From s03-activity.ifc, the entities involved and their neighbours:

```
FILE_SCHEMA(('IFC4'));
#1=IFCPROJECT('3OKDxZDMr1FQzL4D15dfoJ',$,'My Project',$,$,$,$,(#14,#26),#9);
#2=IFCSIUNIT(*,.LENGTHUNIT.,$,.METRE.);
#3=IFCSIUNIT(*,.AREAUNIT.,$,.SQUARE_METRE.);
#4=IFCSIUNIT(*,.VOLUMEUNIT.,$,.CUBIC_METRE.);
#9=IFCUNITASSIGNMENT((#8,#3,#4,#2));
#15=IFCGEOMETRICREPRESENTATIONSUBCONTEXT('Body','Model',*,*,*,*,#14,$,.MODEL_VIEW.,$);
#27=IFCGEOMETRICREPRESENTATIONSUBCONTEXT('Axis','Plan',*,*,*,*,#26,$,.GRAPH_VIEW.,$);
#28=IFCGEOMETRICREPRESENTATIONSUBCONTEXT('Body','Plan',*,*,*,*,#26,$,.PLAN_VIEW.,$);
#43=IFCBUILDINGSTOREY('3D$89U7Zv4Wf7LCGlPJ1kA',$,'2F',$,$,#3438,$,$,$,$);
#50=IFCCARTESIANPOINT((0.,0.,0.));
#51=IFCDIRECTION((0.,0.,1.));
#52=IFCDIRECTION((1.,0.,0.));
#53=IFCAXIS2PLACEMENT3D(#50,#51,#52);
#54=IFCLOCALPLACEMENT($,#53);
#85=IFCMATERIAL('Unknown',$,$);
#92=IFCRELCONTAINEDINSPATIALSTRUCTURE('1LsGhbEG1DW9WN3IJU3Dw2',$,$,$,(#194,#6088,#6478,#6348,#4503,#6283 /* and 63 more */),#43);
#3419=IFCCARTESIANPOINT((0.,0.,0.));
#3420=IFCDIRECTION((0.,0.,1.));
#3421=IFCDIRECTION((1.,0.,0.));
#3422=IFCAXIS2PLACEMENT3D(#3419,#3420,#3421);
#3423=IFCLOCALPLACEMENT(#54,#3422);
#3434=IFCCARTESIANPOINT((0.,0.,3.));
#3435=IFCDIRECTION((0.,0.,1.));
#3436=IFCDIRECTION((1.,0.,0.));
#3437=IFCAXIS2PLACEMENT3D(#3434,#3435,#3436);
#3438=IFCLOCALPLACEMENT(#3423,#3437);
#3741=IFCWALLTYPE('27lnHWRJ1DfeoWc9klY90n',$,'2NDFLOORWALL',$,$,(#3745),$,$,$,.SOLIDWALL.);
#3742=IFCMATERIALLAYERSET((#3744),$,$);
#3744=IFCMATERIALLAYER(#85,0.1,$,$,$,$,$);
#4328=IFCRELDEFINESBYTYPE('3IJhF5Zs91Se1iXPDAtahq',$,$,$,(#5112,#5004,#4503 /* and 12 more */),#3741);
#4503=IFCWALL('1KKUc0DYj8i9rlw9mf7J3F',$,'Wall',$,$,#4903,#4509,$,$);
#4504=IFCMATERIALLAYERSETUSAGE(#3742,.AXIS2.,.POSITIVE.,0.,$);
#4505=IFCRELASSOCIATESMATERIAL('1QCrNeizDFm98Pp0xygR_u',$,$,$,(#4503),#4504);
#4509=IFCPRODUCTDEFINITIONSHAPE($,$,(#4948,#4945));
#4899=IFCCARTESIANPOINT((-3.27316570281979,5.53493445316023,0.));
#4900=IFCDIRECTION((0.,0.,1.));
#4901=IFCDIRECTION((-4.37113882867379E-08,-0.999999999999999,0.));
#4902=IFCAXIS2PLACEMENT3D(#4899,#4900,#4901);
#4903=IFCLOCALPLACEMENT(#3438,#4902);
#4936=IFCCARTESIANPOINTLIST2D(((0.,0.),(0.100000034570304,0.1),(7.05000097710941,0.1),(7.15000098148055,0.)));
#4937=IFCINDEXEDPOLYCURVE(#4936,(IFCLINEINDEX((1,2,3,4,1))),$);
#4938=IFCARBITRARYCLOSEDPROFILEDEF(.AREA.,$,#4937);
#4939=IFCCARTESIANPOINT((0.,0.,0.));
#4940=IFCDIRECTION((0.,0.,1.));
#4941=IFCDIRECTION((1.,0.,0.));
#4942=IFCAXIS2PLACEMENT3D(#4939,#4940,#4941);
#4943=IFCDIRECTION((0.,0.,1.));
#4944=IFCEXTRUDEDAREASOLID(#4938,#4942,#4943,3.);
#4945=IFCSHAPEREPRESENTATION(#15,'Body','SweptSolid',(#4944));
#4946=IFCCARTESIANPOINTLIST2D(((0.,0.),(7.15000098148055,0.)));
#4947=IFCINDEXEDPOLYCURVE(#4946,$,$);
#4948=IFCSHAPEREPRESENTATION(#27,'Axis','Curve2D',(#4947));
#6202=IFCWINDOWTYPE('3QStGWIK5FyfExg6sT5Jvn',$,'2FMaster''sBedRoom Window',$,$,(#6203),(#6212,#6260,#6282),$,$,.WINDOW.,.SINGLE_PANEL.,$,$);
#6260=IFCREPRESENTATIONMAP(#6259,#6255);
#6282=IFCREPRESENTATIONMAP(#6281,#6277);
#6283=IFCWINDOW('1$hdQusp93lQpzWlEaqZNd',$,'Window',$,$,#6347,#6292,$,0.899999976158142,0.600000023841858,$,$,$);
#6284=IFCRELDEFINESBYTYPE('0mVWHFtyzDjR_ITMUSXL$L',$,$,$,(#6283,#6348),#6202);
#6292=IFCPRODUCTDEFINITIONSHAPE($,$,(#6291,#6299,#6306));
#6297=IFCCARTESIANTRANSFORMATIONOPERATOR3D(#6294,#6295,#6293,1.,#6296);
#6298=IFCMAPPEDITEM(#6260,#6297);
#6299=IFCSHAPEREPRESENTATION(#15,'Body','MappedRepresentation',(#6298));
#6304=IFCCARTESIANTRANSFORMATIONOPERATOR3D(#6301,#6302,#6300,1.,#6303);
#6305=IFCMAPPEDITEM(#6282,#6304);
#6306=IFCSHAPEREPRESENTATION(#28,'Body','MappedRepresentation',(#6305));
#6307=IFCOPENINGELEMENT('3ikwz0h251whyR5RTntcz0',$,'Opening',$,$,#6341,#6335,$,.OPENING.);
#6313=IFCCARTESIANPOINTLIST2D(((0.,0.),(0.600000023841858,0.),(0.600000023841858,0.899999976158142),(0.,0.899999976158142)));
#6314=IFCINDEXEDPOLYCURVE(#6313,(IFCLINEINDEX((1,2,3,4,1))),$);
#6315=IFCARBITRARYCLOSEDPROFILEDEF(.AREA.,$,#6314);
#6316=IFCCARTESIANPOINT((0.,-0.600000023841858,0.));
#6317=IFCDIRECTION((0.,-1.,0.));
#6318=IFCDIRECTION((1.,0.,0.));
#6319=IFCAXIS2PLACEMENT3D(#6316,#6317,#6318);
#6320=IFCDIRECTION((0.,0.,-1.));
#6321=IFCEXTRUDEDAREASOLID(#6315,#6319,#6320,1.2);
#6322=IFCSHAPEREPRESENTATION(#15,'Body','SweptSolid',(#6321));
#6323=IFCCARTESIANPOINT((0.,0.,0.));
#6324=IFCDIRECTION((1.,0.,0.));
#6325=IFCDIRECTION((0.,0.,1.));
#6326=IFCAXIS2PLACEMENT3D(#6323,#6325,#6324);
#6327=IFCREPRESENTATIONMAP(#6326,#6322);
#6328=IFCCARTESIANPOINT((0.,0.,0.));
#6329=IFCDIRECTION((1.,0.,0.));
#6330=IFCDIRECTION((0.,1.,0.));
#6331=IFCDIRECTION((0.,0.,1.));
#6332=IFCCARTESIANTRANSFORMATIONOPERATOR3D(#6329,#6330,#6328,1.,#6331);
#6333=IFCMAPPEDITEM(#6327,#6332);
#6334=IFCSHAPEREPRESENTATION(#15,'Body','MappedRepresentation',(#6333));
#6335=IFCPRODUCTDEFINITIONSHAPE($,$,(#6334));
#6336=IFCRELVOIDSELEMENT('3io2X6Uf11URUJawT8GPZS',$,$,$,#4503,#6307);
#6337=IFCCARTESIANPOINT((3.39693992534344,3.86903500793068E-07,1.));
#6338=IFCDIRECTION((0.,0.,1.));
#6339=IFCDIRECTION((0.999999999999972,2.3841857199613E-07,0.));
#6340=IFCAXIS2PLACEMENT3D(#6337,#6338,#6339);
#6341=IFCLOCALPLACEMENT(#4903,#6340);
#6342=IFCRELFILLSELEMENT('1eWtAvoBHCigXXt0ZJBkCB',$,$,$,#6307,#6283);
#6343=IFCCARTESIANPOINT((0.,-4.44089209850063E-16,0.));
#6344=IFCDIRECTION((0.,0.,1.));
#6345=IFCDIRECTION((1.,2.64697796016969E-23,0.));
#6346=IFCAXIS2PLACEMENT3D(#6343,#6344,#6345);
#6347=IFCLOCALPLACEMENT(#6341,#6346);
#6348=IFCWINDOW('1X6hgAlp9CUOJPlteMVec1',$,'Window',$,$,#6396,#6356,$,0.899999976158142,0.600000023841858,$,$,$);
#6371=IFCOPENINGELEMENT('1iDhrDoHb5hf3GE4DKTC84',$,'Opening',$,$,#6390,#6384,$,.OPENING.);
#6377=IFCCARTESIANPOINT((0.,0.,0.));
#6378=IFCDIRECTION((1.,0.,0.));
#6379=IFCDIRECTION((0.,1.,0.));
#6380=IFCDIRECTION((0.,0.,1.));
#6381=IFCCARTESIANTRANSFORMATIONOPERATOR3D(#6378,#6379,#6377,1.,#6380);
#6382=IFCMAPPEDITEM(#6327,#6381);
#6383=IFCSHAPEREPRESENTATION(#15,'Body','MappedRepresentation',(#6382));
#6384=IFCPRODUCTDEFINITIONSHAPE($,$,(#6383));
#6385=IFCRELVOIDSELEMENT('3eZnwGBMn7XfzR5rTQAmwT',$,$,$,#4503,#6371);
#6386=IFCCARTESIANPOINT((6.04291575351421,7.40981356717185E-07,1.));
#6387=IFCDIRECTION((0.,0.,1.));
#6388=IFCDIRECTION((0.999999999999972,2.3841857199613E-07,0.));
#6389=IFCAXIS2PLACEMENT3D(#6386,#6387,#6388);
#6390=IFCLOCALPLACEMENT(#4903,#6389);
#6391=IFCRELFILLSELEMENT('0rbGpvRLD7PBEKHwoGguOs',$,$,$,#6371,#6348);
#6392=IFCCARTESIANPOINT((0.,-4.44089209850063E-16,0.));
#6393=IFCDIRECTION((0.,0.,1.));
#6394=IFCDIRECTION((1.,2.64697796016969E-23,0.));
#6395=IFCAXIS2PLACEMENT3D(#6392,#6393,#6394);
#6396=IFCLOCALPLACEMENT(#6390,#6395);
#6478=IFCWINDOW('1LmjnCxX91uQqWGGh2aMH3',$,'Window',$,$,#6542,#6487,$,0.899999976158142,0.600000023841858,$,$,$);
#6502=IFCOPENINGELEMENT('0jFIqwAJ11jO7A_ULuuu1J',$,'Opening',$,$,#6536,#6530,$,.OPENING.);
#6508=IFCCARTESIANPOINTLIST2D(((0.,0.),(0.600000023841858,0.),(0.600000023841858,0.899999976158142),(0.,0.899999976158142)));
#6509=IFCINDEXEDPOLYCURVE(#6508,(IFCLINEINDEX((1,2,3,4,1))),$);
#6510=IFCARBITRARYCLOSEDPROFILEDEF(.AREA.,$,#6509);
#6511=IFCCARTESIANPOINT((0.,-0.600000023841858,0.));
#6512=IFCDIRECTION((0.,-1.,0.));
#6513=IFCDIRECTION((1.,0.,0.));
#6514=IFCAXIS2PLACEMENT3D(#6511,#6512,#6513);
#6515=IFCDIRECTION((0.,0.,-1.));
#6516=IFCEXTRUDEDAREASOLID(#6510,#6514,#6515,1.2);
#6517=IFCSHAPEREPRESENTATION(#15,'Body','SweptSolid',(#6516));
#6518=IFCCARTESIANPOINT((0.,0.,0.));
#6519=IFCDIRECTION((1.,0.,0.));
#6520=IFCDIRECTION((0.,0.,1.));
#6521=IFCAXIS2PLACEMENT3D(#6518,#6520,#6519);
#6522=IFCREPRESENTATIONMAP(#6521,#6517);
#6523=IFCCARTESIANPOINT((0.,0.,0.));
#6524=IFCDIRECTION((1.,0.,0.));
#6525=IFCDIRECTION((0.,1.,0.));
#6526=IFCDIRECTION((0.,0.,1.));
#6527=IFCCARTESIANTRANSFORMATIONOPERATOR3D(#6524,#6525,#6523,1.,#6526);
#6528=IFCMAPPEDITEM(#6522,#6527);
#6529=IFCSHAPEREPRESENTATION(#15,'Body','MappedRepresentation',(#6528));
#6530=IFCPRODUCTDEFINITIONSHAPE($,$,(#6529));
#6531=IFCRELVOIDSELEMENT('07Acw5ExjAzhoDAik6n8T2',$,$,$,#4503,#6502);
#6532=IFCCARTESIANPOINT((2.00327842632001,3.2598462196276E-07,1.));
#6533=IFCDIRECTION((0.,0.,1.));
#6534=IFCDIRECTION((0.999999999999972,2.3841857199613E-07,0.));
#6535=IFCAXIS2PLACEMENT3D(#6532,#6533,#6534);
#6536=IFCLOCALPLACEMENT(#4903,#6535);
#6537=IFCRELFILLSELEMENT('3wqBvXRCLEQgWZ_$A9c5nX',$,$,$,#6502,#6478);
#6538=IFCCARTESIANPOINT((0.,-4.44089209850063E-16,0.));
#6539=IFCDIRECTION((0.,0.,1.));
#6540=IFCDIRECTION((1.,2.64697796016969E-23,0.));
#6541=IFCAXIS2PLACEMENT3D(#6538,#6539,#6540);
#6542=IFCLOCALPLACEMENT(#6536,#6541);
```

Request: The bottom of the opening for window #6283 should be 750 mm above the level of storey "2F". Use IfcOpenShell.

```python
import numpy as np
import ifcopenshell
import ifcopenshell.api.geometry
import ifcopenshell.geom
import ifcopenshell.util.element
import ifcopenshell.util.placement
import ifcopenshell.util.shape
import ifcopenshell.util.unit

model = ifcopenshell.open("s03-activity.ifc")
unit_scale = ifcopenshell.util.unit.calculate_unit_scale(model)

window = model.by_guid("1$hdQusp93lQpzWlEaqZNd")
opening = window.FillsVoids[0].RelatingOpeningElement
storey = ifcopenshell.util.element.get_container(window, ifc_class="IfcBuildingStorey")
level = ifcopenshell.util.placement.get_local_placement(storey.ObjectPlacement)[2, 3]

# The opening's origin need not be at the sill, so measure its lowest point.
shape = ifcopenshell.geom.create_shape(ifcopenshell.geom.settings(), opening)
bottom = ifcopenshell.util.shape.get_shape_bottom_elevation(shape, shape.geometry) / unit_scale
dz = level + 0.75 / unit_scale - bottom

shift = np.array([0.0, 0.0, dz])
# The window is placed relative to its opening, so it follows when the opening moves.
matrix = ifcopenshell.util.placement.get_local_placement(opening.ObjectPlacement)
matrix[:3, 3] += shift
ifcopenshell.api.geometry.edit_object_placement(
    model, product=opening, matrix=matrix, is_si=False, should_transform_children=True
)

print(f"moved by {dz * unit_scale:+.3f} m")

model.write("s03-activity_v2.ifc")
```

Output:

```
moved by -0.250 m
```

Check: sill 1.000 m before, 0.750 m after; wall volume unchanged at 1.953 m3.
